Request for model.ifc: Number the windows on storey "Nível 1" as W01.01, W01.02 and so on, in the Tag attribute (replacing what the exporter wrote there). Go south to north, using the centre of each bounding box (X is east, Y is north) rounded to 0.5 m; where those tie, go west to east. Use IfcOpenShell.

First a look at what the model holds.

```python
import ifcopenshell
import ifcopenshell.util.element
import ifcopenshell.util.placement

model = ifcopenshell.open("model.ifc")
print(model.schema)
storey = next(s for s in model.by_type("IfcBuildingStorey") if s.Name == "Nível 1")
windows = [e for e in ifcopenshell.util.element.get_decomposition(storey) if e.is_a("IfcWindow")]
for e in sorted(windows, key=lambda e: e.id()):
    origin = ifcopenshell.util.placement.get_local_placement(e.ObjectPlacement)[:3, 3]
    print(e.id(), e.Tag, e.Name, origin.round(2) + 0.0, sep=" | ")
```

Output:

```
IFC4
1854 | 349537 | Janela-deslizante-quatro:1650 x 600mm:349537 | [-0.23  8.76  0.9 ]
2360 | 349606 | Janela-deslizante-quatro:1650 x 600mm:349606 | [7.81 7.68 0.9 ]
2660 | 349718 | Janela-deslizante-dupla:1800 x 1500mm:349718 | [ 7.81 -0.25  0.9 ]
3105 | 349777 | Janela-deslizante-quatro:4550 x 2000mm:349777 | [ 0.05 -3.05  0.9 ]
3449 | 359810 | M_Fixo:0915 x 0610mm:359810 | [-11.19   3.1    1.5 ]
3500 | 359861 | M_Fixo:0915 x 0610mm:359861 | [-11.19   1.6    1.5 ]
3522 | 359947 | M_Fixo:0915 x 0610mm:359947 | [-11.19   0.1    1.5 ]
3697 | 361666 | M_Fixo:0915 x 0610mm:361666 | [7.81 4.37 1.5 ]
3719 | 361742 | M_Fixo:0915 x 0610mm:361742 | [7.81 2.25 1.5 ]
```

```python
import ifcopenshell
import ifcopenshell.geom
import ifcopenshell.util.element
import ifcopenshell.util.shape

model = ifcopenshell.open("model.ifc")
settings = ifcopenshell.geom.settings()
settings.set("use-world-coords", True)


def centre(element):
    shape = ifcopenshell.geom.create_shape(settings, element)
    return ifcopenshell.util.shape.get_bbox_centroid(shape.geometry)


storey = next(s for s in model.by_type("IfcBuildingStorey") if s.Name == "Nível 1")
windows = [e for e in ifcopenshell.util.element.get_decomposition(storey) if e.is_a("IfcWindow")]

# Insertion points can sit at a corner or the storey origin, so sort by the geometry (in metres).
centres = {e: centre(e) for e in windows}
windows.sort(key=lambda e: (round(centres[e][1] / 0.5), centres[e][0]))

for i, e in enumerate(windows, start=1):
    number = f"W01.{i:02d}"
    e.Tag = number
    print(e.id(), number)

model.write("model-out.ifc")
```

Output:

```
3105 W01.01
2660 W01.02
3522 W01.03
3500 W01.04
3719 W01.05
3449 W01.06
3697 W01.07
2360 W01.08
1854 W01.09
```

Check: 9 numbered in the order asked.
